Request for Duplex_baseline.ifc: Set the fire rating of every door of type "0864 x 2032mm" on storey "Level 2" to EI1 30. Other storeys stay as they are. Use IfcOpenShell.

First a look at what the model holds.

```python
import ifcopenshell
import ifcopenshell.util.element

model = ifcopenshell.open("Duplex_baseline.ifc")
print(model.schema)
storey = next(s for s in model.by_type("IfcBuildingStorey") if s.Name == "Level 2")
doors = [e for e in ifcopenshell.util.element.get_decomposition(storey) if e.is_a("IfcDoor")]
seen = {}
for e in doors:
    element_type = ifcopenshell.util.element.get_type(e)
    key = (element_type.Name if element_type != e and element_type else None, ifcopenshell.util.element.get_pset(e, "Pset_DoorCommon", "FireRating"))
    seen[key] = seen.get(key, 0) + 1
for (name, value), count in sorted(seen.items(), key=str):
    print(count, "x", name, "|", value)
```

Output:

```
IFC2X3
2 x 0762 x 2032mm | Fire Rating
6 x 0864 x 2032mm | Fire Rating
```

```python
import ifcopenshell
import ifcopenshell.api.pset
import ifcopenshell.util.element

model = ifcopenshell.open("Duplex_baseline.ifc")

storey = next(s for s in model.by_type("IfcBuildingStorey") if s.Name == "Level 2")
doors = [e for e in ifcopenshell.util.element.get_decomposition(storey) if e.is_a("IfcDoor")]

count = 0
for e in doors:
    element_type = ifcopenshell.util.element.get_type(e)
    if element_type in (None, e) or element_type.Name != "0864 x 2032mm":
        continue
    # add_pset returns the element's existing set when there is one.
    pset = ifcopenshell.api.pset.add_pset(model, product=e, name="Pset_DoorCommon")
    ifcopenshell.api.pset.edit_pset(model, pset=pset, properties={"FireRating": "EI1 30"})
    count += 1

print(count, "doors updated")

model.write("Duplex_baseline_edited.ifc")
```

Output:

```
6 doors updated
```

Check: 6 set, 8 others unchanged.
